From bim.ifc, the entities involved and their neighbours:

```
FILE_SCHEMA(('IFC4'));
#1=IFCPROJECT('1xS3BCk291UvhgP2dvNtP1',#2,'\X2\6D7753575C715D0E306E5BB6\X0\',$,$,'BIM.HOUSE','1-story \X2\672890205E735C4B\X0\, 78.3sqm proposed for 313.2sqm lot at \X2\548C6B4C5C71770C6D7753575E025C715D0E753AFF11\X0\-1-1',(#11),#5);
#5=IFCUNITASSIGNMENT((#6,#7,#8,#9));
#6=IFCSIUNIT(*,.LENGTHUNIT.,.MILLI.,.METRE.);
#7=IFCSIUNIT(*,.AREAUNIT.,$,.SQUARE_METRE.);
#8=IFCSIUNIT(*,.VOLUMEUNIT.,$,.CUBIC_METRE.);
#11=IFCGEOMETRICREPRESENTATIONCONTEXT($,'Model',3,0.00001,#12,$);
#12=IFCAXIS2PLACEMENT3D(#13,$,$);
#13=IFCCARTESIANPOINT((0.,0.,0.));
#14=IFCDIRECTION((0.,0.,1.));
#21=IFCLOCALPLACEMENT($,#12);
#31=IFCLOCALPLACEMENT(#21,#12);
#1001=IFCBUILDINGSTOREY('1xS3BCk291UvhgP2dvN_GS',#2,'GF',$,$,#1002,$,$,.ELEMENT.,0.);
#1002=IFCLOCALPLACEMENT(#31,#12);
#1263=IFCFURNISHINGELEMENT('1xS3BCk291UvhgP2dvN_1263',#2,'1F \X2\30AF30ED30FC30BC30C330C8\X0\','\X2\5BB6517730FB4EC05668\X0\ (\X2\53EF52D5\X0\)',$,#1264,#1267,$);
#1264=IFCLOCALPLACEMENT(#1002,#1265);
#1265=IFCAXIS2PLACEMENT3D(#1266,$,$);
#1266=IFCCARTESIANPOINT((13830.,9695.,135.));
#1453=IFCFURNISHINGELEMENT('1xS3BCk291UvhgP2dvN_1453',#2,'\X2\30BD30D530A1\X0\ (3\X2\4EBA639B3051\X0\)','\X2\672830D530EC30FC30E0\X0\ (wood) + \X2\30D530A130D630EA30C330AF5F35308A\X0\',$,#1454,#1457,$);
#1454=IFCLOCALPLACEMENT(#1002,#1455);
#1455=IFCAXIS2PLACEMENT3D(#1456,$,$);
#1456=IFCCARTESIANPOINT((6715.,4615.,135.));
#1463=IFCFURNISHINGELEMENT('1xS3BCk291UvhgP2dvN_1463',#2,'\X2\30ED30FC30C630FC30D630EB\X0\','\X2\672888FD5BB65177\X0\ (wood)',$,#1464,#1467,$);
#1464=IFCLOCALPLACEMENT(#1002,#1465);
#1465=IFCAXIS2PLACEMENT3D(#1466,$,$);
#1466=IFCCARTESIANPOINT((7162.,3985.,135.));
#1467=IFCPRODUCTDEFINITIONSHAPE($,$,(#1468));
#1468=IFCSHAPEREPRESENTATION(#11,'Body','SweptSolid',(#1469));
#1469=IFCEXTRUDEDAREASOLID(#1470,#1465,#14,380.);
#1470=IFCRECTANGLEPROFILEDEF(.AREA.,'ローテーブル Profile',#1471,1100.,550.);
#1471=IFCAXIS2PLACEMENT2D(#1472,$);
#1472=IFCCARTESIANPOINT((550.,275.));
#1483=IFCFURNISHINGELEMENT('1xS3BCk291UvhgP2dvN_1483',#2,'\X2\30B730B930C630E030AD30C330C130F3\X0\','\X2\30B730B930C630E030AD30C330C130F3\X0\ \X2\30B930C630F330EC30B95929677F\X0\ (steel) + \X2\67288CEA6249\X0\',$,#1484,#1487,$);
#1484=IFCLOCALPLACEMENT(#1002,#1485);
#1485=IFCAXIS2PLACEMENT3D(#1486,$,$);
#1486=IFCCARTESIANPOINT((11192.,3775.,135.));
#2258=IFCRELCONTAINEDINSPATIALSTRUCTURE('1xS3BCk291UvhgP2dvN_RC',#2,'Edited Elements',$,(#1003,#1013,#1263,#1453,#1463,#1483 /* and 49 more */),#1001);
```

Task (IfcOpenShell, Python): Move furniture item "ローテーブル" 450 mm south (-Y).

```python
import ifcopenshell
import ifcopenshell.api.geometry
import ifcopenshell.util.placement
import ifcopenshell.util.unit

model = ifcopenshell.open("bim.ifc")
unit_scale = ifcopenshell.util.unit.calculate_unit_scale(model)

item = model.by_id(1463)
matrix = ifcopenshell.util.placement.get_local_placement(item.ObjectPlacement)
matrix[1, 3] -= 0.45 / unit_scale
ifcopenshell.api.geometry.edit_object_placement(model, product=item, matrix=matrix, is_si=False)

print(ifcopenshell.util.placement.get_local_placement(item.ObjectPlacement).round(3) + 0.0)

model.write("bim_v2.ifc")
```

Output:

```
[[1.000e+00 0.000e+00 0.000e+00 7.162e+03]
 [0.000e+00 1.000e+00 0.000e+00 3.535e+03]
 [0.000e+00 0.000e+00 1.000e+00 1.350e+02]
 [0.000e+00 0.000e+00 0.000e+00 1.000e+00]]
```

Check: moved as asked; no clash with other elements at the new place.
